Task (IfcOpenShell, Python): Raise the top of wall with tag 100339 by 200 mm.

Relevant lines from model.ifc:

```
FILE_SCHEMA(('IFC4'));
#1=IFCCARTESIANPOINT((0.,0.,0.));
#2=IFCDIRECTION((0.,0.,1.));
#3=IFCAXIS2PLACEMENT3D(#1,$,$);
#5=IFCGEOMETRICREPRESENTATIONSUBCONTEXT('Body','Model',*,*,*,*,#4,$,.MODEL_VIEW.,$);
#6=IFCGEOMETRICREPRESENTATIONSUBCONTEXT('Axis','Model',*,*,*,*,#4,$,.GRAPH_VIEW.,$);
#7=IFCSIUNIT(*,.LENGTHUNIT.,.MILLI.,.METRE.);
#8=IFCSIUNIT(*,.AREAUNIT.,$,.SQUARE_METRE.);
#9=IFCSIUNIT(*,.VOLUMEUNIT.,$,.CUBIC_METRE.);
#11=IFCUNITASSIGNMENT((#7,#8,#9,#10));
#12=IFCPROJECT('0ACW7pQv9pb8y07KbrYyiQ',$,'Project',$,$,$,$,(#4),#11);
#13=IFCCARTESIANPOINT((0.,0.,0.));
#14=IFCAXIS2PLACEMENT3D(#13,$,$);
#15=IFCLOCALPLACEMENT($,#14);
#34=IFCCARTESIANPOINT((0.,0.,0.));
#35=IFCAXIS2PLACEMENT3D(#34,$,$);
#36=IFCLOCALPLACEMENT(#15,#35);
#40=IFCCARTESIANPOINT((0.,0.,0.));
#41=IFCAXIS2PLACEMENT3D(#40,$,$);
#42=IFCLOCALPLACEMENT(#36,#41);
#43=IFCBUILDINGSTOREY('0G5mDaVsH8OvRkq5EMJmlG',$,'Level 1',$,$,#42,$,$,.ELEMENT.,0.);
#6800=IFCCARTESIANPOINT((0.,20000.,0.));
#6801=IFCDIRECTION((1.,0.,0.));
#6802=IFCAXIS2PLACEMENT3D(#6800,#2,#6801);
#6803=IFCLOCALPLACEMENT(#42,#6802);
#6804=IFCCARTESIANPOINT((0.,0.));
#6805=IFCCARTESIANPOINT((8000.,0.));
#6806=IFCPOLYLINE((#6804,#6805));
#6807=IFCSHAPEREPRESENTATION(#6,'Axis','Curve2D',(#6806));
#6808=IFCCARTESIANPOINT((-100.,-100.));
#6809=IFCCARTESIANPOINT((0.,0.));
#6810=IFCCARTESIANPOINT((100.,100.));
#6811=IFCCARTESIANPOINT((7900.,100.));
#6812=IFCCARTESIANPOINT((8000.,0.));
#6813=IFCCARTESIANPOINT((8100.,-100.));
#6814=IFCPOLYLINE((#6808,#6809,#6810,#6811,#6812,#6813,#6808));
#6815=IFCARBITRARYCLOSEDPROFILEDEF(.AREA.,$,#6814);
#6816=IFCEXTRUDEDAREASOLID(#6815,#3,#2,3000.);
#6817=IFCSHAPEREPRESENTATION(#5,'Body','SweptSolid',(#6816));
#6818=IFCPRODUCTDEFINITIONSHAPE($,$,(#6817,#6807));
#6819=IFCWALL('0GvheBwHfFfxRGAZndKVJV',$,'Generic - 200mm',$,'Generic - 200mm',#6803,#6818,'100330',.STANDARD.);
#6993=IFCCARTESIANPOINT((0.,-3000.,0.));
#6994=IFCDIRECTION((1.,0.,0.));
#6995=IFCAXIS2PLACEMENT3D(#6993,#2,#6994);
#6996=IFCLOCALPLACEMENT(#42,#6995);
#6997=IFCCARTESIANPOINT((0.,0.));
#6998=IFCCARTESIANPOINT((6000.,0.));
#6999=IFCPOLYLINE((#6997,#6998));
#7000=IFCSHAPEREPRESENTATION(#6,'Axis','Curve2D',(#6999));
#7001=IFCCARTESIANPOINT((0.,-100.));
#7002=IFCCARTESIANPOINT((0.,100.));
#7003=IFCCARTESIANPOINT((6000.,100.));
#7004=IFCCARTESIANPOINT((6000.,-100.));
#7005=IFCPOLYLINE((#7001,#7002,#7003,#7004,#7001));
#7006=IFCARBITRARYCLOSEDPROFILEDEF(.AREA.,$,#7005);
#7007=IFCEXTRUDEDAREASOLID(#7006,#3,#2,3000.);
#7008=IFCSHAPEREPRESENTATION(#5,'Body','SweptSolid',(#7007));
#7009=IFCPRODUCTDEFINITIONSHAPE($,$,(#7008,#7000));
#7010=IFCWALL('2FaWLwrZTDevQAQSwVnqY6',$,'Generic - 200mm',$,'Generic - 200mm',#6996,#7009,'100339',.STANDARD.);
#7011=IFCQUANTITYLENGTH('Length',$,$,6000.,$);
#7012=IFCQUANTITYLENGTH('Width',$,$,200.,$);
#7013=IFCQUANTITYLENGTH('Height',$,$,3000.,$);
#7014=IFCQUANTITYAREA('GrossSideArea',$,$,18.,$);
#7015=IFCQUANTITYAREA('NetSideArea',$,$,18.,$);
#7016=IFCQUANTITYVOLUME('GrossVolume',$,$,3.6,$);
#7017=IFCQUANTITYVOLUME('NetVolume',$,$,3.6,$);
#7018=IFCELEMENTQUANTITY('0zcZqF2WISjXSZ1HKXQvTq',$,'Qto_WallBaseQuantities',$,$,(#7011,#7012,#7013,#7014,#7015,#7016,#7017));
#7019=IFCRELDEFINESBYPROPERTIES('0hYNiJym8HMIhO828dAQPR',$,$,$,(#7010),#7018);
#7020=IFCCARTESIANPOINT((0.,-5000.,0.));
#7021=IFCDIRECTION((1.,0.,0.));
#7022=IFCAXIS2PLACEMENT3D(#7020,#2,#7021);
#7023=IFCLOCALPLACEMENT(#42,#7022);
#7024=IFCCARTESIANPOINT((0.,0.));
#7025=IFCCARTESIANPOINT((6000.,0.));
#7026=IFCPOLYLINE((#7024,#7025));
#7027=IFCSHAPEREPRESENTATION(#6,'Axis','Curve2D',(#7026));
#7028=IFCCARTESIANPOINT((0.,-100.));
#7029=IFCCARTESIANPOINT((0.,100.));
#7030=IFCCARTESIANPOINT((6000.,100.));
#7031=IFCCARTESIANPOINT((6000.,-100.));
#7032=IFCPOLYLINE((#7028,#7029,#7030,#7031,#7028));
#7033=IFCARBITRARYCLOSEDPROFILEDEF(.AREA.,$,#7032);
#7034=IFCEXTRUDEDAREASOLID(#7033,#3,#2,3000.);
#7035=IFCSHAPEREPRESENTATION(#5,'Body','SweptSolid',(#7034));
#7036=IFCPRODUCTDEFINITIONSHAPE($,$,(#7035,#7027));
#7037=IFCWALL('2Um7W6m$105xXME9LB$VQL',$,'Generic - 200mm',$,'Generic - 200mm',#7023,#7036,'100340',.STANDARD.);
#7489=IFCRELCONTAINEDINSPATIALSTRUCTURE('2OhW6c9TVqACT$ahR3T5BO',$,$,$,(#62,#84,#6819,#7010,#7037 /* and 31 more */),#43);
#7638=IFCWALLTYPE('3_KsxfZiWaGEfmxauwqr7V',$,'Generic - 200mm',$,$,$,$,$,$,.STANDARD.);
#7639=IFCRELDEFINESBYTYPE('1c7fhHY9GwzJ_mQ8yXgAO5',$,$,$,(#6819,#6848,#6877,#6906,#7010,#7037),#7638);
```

```python
import ifcopenshell
import ifcopenshell.api.pset
import ifcopenshell.geom
import ifcopenshell.util.element
import ifcopenshell.util.representation
import ifcopenshell.util.shape
import ifcopenshell.util.unit

model = ifcopenshell.open("model.ifc")
unit_scale = ifcopenshell.util.unit.calculate_unit_scale(model)
area_scale = ifcopenshell.util.unit.calculate_unit_scale(model, "AREAUNIT")
volume_scale = ifcopenshell.util.unit.calculate_unit_scale(model, "VOLUMEUNIT")
settings = ifcopenshell.geom.settings()


def volume(element):
    """Net volume in cubic metres, openings subtracted."""
    shape = ifcopenshell.geom.create_shape(settings, element)
    return ifcopenshell.util.shape.get_volume(shape.geometry)


wall = model.by_id(7010)
before = volume(wall)

body = ifcopenshell.util.representation.get_representation(wall, "Model", "Body")
solid = body.Items[0]
old_height = solid.Depth
solid.Depth += 200.0
after = volume(wall)
thickness = 0.2  # wall thickness in metres

# Update the stored height, areas and volumes.
qto = model.by_id(ifcopenshell.util.element.get_pset(wall, "Qto_WallBaseQuantities", should_inherit=False)["id"])
ifcopenshell.api.pset.edit_qto(model, qto=qto, properties={
    "Height": solid.Depth,
    "GrossSideArea": ifcopenshell.util.element.get_pset(wall, "Qto_WallBaseQuantities", "GrossSideArea") * solid.Depth / old_height,
    "NetSideArea": after / thickness / area_scale,
    "GrossVolume": ifcopenshell.util.element.get_pset(wall, "Qto_WallBaseQuantities", "GrossVolume") * solid.Depth / old_height,
    "NetVolume": after / volume_scale,
})

print(f"height {old_height:g} -> {solid.Depth:g}, volume {before:.3f} -> {after:.3f} m3")

model.write("model-out.ifc")
```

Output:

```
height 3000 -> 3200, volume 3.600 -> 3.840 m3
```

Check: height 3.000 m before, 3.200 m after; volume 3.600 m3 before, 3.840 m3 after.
